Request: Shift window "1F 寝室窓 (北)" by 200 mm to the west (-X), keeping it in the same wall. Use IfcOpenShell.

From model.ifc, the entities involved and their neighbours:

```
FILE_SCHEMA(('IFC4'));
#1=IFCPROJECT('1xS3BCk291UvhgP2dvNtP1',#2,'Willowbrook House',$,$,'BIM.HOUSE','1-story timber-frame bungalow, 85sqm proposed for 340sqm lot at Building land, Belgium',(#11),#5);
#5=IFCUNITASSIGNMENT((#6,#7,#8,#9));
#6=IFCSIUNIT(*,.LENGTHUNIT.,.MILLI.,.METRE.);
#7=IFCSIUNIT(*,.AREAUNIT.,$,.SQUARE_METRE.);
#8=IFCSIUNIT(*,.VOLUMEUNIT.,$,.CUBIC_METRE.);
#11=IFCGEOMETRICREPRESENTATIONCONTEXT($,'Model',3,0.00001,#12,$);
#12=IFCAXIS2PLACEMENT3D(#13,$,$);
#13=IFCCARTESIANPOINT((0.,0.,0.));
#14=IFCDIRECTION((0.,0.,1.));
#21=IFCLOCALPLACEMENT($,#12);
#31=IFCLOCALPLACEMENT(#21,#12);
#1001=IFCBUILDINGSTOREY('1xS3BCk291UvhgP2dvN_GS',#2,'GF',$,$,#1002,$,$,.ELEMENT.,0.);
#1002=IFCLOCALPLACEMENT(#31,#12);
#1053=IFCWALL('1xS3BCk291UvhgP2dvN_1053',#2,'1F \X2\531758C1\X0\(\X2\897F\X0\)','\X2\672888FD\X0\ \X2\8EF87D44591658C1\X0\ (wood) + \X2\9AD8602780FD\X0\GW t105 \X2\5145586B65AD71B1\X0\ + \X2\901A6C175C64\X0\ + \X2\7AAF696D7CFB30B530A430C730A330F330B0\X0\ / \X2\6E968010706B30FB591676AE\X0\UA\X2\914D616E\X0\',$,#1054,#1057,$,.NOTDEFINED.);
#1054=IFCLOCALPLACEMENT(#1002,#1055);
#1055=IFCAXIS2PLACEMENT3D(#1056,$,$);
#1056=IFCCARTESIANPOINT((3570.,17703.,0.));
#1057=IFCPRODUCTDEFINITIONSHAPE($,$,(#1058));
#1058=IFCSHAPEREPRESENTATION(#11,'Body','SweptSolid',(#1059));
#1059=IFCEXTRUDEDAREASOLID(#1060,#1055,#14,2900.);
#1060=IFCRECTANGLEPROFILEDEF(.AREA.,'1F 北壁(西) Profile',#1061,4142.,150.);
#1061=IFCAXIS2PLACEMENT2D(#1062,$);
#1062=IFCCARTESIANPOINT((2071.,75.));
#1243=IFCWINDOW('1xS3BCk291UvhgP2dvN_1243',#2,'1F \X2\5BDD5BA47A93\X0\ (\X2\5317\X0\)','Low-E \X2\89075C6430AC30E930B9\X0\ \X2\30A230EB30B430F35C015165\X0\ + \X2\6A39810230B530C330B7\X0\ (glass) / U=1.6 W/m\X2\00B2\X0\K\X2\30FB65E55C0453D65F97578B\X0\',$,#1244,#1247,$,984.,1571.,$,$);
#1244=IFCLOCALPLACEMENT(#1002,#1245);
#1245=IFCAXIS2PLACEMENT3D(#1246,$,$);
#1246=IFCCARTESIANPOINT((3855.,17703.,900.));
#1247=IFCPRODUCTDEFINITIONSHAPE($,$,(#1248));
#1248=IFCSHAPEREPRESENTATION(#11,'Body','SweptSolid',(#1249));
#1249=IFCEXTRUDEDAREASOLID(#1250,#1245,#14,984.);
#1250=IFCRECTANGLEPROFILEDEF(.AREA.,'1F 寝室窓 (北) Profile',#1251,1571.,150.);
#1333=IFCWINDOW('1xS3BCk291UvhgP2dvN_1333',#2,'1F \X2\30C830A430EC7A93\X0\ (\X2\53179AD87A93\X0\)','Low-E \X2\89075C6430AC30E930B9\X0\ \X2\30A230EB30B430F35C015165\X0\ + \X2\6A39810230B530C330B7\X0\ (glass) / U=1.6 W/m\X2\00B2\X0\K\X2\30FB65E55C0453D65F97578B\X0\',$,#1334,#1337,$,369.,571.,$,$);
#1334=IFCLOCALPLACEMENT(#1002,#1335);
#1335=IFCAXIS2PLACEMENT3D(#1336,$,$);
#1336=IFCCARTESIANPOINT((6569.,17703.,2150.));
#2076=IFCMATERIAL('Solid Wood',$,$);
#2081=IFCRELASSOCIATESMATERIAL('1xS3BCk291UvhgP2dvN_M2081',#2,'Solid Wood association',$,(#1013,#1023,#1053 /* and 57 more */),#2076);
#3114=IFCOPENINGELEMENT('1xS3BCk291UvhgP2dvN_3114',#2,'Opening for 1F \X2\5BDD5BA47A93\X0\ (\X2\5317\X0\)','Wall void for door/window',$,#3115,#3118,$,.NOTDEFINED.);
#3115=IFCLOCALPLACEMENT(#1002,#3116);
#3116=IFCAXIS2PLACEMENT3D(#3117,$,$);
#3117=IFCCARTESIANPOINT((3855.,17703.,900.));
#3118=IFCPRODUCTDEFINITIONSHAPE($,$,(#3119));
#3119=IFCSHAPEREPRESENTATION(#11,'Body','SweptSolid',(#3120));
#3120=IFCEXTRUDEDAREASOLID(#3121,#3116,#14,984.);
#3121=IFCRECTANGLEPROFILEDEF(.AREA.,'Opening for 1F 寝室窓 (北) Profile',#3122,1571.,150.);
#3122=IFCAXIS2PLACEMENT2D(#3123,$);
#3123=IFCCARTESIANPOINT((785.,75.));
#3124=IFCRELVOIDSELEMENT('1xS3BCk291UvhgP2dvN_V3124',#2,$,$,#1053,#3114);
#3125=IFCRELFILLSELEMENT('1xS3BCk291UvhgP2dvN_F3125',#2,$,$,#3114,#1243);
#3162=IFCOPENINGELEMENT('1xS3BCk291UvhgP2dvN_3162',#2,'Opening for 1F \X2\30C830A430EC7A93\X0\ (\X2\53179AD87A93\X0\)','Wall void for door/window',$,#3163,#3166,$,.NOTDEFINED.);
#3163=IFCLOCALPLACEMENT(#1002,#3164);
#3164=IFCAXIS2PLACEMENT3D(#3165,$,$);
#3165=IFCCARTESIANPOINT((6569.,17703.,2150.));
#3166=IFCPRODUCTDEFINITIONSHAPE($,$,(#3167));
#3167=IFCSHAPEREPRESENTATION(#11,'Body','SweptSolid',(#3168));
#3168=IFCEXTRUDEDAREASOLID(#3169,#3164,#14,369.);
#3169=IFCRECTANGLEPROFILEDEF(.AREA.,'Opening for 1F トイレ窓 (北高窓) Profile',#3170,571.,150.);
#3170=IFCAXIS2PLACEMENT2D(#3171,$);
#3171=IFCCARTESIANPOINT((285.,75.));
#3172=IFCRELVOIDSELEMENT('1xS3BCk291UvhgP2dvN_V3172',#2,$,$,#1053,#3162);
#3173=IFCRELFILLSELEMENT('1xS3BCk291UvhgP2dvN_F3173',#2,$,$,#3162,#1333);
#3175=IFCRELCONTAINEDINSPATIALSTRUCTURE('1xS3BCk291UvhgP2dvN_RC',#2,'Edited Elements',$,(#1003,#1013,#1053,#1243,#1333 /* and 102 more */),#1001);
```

```python
import ifcopenshell
import ifcopenshell.api.geometry
import ifcopenshell.util.placement

model = ifcopenshell.open("model.ifc")

window = model.by_guid("1xS3BCk291UvhgP2dvN_1243")
opening = window.FillsVoids[0].RelatingOpeningElement
wall = opening.VoidsElements[0].RelatingBuildingElement

wall_matrix = ifcopenshell.util.placement.get_local_placement(wall.ObjectPlacement)
shift = wall_matrix[:3, 0] * -200.0
before = ifcopenshell.util.placement.get_local_placement(window.ObjectPlacement)[:3, 3].copy()

# The window is not placed relative to its opening, so move both.
for product in (opening, window):
    matrix = ifcopenshell.util.placement.get_local_placement(product.ObjectPlacement)
    matrix[:3, 3] += shift
    ifcopenshell.api.geometry.edit_object_placement(model, product=product, matrix=matrix, is_si=False)

after = ifcopenshell.util.placement.get_local_placement(window.ObjectPlacement)[:3, 3]
print("window moved by", (after - before).round(3) + 0.0)

model.write("model_v2.ifc")
```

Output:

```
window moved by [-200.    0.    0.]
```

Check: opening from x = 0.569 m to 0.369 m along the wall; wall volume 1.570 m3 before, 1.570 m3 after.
